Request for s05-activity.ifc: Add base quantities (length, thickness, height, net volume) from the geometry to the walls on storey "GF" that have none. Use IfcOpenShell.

First a look at what the model holds.

```python
import ifcopenshell
import ifcopenshell.util.element
import ifcopenshell.util.unit

model = ifcopenshell.open("s05-activity.ifc")
print(model.schema)
for unit_type in ("LENGTHUNIT", "AREAUNIT", "VOLUMEUNIT"):
    print(unit_type, ifcopenshell.util.unit.calculate_unit_scale(model, unit_type))
storey = next(s for s in model.by_type("IfcBuildingStorey") if s.Name == "GF")
walls = [e for e in ifcopenshell.util.element.get_decomposition(storey) if e.is_a("IfcWall")]
for e in sorted(walls, key=lambda e: e.id()):
    print(e.id(), e.is_a(), e.Name, list(ifcopenshell.util.element.get_psets(e, qtos_only=True)), sep=" | ")
```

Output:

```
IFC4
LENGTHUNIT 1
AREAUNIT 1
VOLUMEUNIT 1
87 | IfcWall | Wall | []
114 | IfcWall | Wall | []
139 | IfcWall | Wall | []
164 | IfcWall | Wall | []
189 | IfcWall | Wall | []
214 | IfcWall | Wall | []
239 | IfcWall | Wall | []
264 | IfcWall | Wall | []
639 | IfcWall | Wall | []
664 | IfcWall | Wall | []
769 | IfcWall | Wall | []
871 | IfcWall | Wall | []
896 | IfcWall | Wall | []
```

```python
import ifcopenshell
import ifcopenshell.api.pset
import ifcopenshell.geom
import ifcopenshell.util.element
import ifcopenshell.util.shape
import ifcopenshell.util.unit

model = ifcopenshell.open("s05-activity.ifc")
unit_scale = ifcopenshell.util.unit.calculate_unit_scale(model)
volume_scale = ifcopenshell.util.unit.calculate_unit_scale(model, "VOLUMEUNIT")
settings = ifcopenshell.geom.settings()

storey = next(s for s in model.by_type("IfcBuildingStorey") if s.Name == "GF")
walls = [e for e in ifcopenshell.util.element.get_decomposition(storey) if e.is_a("IfcWall")]

for e in sorted(walls, key=lambda e: e.id()):
    if ifcopenshell.util.element.get_psets(e, qtos_only=True, should_inherit=False):
        continue
    # Geometry comes back in metres, in the element's own axes.
    shape = ifcopenshell.geom.create_shape(settings, e)
    values = {
        "Length": ifcopenshell.util.shape.get_x(shape.geometry) / unit_scale,
        "Width": ifcopenshell.util.shape.get_y(shape.geometry) / unit_scale,
        "Height": ifcopenshell.util.shape.get_z(shape.geometry) / unit_scale,
        "NetVolume": ifcopenshell.util.shape.get_volume(shape.geometry) / volume_scale,
    }
    qto = ifcopenshell.api.pset.add_qto(model, product=e, name="Qto_WallBaseQuantities")
    ifcopenshell.api.pset.edit_qto(model, qto=qto, properties=values)
    print(e.id(), {k: round(v, 3) for k, v in values.items()})

model.write("s05-activity_updated.ifc")
```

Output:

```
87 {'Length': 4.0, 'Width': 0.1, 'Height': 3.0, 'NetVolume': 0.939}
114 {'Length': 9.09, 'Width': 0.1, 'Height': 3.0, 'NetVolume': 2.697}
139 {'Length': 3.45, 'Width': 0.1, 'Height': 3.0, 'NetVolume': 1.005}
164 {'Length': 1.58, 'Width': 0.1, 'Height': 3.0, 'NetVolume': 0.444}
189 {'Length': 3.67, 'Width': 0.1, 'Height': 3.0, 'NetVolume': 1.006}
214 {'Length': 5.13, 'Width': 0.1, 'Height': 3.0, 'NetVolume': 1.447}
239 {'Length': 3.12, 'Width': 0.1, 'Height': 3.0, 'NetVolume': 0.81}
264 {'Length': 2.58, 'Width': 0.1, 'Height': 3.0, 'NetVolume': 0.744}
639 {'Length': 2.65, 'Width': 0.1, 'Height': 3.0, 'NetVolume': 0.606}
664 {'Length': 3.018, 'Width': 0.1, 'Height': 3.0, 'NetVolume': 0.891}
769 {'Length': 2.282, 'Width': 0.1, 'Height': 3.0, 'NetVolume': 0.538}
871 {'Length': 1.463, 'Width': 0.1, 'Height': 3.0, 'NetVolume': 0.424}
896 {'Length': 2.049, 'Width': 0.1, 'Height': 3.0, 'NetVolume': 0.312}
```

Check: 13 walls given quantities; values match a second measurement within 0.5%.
